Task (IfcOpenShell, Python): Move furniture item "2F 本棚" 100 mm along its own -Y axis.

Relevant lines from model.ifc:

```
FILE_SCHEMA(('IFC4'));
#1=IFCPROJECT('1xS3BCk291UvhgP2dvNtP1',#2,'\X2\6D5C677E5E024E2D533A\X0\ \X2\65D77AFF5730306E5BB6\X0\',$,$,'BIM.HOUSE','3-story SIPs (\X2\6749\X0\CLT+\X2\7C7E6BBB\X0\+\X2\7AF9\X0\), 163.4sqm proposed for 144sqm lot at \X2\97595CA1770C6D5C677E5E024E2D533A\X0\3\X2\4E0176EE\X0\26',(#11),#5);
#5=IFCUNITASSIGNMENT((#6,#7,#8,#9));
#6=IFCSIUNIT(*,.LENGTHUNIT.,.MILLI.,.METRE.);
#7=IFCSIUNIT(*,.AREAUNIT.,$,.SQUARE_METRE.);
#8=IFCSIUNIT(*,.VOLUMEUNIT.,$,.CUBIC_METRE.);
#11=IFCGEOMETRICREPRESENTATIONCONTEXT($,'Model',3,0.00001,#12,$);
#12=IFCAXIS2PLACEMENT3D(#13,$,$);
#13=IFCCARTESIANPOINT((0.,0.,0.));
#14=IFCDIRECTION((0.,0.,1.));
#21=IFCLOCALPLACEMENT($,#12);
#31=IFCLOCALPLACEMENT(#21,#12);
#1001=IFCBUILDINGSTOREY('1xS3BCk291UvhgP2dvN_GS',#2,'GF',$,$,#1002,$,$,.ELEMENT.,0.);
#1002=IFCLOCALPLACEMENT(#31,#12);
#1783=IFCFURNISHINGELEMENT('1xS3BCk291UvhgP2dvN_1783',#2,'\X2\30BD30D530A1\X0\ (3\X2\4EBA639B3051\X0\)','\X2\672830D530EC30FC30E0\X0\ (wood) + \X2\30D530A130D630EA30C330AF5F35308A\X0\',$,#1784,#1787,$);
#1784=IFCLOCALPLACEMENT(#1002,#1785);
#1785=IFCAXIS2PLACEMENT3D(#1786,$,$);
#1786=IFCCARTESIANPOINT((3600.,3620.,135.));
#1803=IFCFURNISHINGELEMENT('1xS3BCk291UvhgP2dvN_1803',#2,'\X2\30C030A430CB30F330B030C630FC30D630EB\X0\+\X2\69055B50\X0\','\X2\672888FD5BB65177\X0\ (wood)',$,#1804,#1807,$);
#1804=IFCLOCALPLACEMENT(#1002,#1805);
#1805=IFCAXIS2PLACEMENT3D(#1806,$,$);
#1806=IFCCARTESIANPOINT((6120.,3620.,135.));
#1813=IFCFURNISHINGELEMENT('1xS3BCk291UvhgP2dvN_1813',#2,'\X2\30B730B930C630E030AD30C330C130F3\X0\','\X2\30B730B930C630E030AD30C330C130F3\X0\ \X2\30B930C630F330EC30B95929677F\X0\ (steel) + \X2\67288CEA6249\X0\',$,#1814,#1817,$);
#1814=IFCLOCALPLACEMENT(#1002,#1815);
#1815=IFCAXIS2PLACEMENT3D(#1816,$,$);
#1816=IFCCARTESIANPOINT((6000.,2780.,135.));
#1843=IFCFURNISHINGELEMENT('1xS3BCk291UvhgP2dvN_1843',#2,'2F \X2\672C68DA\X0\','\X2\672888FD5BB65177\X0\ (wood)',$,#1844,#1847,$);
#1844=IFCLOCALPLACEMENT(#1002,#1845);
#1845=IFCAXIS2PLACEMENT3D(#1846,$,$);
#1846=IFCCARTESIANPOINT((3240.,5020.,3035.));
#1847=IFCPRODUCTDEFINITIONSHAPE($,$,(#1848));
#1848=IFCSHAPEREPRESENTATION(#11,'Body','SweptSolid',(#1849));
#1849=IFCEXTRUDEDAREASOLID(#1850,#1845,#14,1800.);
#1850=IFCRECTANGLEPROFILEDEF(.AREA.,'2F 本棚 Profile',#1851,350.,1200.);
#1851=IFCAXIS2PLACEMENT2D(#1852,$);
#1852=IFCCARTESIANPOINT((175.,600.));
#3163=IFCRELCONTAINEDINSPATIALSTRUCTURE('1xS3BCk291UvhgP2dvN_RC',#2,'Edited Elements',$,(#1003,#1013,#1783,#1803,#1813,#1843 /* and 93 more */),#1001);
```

```python
import ifcopenshell
import ifcopenshell.api.geometry
import ifcopenshell.util.placement
import ifcopenshell.util.unit

model = ifcopenshell.open("model.ifc")
unit_scale = ifcopenshell.util.unit.calculate_unit_scale(model)

item = model.by_guid("1xS3BCk291UvhgP2dvN_1843")
matrix = ifcopenshell.util.placement.get_local_placement(item.ObjectPlacement)
matrix[:3, 3] -= matrix[:3, 1] * 0.1 / unit_scale
ifcopenshell.api.geometry.edit_object_placement(model, product=item, matrix=matrix, is_si=False)

print(ifcopenshell.util.placement.get_local_placement(item.ObjectPlacement).round(3) + 0.0)

model.write("model-out.ifc")
```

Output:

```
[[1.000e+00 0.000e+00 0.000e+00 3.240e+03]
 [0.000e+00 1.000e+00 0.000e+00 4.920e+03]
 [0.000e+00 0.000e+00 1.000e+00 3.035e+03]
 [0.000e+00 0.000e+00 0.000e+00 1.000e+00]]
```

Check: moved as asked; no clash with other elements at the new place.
